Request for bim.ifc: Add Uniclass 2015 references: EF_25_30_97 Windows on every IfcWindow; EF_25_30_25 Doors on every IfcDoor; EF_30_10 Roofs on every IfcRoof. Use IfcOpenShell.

First a look at what the model holds.

```python
import ifcopenshell

model = ifcopenshell.open("bim.ifc")
print(model.schema)
print("classifications:", [c.Name for c in model.by_type("IfcClassification")])
for ifc_class in ("IfcDoor", "IfcRoof", "IfcStair", "IfcWall", "IfcWindow"):
    print(ifc_class, len(model.by_type(ifc_class)))
```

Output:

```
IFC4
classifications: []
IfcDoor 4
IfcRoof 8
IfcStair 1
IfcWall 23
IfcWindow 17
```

```python
import ifcopenshell
import ifcopenshell.api.classification

model = ifcopenshell.open("bim.ifc")

system = ifcopenshell.api.classification.add_classification(model, classification="Uniclass 2015")

codes = {
    "IfcWindow": ("EF_25_30_97", "Windows"),
    "IfcDoor": ("EF_25_30_25", "Doors"),
    "IfcRoof": ("EF_30_10", "Roofs"),
}
for ifc_class, (code, name) in codes.items():
    products = model.by_type(ifc_class)
    ifcopenshell.api.classification.add_reference(
        model, products=products, classification=system, identification=code, name=name
    )
    print(code, len(products))

model.write("bim_v2.ifc")
```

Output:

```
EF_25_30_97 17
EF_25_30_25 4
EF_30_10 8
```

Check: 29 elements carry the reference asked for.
